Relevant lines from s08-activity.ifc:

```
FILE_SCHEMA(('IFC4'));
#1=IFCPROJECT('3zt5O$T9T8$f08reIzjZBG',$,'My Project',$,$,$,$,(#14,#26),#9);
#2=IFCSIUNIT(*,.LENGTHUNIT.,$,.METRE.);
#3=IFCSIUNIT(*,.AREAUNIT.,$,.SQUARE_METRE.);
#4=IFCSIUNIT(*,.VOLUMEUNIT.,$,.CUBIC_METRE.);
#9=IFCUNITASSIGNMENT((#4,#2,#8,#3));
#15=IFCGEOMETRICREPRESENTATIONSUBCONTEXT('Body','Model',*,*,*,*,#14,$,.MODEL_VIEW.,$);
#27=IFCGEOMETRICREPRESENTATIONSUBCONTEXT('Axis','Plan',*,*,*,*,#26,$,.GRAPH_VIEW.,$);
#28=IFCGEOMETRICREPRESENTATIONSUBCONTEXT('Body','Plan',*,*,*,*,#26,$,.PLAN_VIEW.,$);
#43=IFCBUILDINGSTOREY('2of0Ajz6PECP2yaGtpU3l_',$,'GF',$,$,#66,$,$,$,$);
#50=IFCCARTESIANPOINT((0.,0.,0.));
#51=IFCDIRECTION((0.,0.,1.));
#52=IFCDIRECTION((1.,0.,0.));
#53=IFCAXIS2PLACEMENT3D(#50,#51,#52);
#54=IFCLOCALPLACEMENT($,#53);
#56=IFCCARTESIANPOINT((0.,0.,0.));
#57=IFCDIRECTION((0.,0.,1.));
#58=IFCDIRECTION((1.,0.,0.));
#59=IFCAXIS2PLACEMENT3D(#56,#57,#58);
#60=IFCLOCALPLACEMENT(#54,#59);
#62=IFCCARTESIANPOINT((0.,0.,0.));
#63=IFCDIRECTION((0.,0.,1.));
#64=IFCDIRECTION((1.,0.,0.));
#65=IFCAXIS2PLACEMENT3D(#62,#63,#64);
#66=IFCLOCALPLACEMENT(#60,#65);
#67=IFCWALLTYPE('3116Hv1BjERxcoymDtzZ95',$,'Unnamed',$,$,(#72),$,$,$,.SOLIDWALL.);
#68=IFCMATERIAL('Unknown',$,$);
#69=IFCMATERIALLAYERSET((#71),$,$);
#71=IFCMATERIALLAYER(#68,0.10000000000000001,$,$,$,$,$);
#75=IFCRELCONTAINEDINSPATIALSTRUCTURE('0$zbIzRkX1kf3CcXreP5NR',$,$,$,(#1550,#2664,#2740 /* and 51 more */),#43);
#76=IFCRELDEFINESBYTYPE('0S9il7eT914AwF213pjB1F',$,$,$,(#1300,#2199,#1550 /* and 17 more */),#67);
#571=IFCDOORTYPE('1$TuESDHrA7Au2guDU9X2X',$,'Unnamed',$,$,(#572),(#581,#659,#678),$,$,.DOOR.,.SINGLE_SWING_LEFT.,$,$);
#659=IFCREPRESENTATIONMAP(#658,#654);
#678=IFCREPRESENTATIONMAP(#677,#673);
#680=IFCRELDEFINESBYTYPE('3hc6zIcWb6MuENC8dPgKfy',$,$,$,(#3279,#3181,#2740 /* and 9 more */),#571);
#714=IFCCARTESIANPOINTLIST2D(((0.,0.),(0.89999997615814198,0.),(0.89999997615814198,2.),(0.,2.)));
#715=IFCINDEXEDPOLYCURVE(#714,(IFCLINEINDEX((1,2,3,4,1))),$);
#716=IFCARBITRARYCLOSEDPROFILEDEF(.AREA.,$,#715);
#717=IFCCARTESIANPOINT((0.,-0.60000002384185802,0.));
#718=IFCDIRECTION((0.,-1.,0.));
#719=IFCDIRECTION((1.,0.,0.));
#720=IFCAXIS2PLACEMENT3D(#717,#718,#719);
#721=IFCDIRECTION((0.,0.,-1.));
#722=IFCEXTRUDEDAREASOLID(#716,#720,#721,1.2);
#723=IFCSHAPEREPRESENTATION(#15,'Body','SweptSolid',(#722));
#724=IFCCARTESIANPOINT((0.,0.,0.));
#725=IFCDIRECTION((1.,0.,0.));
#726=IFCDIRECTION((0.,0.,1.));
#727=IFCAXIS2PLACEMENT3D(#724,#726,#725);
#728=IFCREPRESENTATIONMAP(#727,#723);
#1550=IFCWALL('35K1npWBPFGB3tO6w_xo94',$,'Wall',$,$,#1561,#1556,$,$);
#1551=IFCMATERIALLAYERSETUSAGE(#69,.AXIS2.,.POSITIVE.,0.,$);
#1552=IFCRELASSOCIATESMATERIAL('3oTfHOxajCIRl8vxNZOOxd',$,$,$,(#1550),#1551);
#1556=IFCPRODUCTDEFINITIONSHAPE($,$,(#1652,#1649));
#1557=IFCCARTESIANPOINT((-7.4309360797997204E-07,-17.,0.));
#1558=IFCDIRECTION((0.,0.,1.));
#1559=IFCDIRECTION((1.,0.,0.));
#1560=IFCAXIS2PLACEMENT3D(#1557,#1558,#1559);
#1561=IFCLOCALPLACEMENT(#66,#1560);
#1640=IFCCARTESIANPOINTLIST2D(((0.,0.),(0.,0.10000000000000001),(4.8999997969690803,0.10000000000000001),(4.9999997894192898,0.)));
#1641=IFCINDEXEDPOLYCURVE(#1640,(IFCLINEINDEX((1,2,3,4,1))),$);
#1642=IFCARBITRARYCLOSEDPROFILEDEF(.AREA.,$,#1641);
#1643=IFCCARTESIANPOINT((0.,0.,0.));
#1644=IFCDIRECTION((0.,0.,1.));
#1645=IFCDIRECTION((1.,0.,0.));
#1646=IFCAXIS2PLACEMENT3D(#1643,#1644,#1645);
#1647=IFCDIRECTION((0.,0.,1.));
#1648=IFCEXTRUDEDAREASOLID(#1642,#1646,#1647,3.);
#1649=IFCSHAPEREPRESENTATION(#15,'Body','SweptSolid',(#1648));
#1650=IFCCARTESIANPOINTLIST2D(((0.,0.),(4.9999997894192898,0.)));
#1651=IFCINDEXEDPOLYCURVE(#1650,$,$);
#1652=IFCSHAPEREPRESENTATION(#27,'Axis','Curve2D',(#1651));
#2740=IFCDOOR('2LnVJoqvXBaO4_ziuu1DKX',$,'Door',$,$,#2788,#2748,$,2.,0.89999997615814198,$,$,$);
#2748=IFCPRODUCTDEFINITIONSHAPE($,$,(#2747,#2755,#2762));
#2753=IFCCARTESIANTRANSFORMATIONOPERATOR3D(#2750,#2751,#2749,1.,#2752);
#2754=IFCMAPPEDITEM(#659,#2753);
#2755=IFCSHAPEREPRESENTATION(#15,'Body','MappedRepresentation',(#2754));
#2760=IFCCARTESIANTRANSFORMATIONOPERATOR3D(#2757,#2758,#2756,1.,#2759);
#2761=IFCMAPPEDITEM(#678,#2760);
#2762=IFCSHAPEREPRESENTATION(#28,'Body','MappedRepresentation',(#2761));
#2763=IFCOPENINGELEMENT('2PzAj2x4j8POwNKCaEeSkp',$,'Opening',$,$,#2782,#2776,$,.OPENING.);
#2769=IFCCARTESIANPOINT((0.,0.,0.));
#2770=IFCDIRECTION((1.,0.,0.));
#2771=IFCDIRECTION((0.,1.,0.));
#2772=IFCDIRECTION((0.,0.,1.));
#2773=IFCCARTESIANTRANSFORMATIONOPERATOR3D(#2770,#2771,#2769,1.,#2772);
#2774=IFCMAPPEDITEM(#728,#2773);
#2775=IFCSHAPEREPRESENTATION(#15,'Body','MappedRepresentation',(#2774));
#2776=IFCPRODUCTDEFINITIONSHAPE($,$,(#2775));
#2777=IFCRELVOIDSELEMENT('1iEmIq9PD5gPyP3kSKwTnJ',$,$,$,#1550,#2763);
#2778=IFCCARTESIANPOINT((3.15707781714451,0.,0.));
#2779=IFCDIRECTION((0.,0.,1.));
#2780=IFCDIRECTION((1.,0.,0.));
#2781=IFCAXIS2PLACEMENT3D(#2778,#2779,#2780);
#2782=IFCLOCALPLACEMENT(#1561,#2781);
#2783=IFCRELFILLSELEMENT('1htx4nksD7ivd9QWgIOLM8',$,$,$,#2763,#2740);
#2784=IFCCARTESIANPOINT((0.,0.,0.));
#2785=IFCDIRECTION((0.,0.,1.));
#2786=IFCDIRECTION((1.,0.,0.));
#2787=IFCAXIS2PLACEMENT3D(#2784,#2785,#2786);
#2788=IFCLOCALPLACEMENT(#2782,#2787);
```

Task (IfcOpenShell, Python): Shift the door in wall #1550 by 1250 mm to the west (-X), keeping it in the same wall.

```python
import ifcopenshell
import ifcopenshell.api.geometry
import ifcopenshell.util.placement

model = ifcopenshell.open("s08-activity.ifc")

door = model.by_guid("2LnVJoqvXBaO4_ziuu1DKX")
opening = door.FillsVoids[0].RelatingOpeningElement
wall = opening.VoidsElements[0].RelatingBuildingElement

wall_matrix = ifcopenshell.util.placement.get_local_placement(wall.ObjectPlacement)
shift = wall_matrix[:3, 0] * -1.25
before = ifcopenshell.util.placement.get_local_placement(door.ObjectPlacement)[:3, 3].copy()

# The door is placed relative to its opening, so it follows when the opening moves.
matrix = ifcopenshell.util.placement.get_local_placement(opening.ObjectPlacement)
matrix[:3, 3] += shift
ifcopenshell.api.geometry.edit_object_placement(
    model, product=opening, matrix=matrix, is_si=False, should_transform_children=True
)

after = ifcopenshell.util.placement.get_local_placement(door.ObjectPlacement)[:3, 3]
print("door moved by", (after - before).round(3) + 0.0)

model.write("s08-activity_rev.ifc")
```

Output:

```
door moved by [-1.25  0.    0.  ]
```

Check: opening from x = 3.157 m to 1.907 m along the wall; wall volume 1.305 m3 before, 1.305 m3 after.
